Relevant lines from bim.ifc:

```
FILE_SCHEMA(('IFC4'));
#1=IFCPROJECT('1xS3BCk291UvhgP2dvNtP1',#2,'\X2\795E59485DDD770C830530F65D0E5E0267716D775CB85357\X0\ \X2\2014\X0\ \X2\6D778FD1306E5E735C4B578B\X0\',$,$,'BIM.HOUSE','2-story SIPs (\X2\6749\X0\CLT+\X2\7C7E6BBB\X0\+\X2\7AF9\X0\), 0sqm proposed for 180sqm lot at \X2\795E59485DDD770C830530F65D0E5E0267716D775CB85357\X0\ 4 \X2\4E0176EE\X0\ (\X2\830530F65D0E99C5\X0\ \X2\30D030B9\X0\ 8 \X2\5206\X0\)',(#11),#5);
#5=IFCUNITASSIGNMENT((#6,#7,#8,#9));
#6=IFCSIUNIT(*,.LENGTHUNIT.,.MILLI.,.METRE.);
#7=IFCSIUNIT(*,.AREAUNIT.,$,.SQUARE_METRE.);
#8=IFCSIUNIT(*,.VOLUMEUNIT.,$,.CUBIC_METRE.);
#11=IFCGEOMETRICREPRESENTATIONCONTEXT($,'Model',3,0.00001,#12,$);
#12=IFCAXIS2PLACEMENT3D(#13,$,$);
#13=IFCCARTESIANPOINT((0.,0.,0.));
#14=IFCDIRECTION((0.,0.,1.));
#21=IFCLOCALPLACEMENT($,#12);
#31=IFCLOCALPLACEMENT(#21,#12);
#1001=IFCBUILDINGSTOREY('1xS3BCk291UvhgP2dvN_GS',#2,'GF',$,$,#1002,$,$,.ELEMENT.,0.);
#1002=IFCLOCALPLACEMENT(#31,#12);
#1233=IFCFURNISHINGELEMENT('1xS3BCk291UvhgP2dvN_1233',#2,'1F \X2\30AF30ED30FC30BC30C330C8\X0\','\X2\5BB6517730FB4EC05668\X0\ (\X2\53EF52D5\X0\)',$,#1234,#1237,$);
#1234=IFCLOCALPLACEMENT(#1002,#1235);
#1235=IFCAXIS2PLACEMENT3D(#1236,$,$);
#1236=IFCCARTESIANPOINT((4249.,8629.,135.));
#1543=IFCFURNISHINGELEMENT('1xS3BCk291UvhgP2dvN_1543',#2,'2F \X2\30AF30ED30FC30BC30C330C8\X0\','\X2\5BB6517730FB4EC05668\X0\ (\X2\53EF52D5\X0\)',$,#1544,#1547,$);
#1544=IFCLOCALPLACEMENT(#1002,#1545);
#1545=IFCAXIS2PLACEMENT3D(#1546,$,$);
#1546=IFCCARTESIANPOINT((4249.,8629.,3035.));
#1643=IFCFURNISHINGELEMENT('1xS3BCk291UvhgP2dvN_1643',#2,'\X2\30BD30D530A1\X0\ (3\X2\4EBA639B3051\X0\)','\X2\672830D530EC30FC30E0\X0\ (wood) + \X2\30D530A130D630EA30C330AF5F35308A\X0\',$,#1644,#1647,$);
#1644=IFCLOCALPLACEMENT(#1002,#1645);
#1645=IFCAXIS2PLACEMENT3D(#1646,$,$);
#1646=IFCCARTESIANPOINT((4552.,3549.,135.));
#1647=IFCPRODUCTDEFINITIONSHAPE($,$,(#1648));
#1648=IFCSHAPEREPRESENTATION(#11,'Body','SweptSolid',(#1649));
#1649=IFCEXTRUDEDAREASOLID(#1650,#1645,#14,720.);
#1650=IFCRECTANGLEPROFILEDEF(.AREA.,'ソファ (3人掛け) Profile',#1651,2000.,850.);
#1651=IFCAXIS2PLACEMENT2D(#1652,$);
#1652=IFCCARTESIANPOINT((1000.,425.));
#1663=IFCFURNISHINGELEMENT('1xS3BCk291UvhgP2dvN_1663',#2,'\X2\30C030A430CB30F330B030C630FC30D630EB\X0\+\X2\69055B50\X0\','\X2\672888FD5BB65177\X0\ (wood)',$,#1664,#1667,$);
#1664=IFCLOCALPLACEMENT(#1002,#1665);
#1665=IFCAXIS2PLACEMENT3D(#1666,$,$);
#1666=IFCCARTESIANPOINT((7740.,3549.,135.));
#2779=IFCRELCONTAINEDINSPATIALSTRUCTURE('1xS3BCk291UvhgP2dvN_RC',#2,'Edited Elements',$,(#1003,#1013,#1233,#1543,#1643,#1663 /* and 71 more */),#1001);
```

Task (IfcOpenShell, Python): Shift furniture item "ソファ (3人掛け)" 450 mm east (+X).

```python
import ifcopenshell
import ifcopenshell.api.geometry
import ifcopenshell.util.placement
import ifcopenshell.util.unit

model = ifcopenshell.open("bim.ifc")
unit_scale = ifcopenshell.util.unit.calculate_unit_scale(model)

item = model.by_id(1643)
matrix = ifcopenshell.util.placement.get_local_placement(item.ObjectPlacement)
matrix[0, 3] += 0.45 / unit_scale
ifcopenshell.api.geometry.edit_object_placement(model, product=item, matrix=matrix, is_si=False)

print(ifcopenshell.util.placement.get_local_placement(item.ObjectPlacement).round(3) + 0.0)

model.write("bim_v2.ifc")
```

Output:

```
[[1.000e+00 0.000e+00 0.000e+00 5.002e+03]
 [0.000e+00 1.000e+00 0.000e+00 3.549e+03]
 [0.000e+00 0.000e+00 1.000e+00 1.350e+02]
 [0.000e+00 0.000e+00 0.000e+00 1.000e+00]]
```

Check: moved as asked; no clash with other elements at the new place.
